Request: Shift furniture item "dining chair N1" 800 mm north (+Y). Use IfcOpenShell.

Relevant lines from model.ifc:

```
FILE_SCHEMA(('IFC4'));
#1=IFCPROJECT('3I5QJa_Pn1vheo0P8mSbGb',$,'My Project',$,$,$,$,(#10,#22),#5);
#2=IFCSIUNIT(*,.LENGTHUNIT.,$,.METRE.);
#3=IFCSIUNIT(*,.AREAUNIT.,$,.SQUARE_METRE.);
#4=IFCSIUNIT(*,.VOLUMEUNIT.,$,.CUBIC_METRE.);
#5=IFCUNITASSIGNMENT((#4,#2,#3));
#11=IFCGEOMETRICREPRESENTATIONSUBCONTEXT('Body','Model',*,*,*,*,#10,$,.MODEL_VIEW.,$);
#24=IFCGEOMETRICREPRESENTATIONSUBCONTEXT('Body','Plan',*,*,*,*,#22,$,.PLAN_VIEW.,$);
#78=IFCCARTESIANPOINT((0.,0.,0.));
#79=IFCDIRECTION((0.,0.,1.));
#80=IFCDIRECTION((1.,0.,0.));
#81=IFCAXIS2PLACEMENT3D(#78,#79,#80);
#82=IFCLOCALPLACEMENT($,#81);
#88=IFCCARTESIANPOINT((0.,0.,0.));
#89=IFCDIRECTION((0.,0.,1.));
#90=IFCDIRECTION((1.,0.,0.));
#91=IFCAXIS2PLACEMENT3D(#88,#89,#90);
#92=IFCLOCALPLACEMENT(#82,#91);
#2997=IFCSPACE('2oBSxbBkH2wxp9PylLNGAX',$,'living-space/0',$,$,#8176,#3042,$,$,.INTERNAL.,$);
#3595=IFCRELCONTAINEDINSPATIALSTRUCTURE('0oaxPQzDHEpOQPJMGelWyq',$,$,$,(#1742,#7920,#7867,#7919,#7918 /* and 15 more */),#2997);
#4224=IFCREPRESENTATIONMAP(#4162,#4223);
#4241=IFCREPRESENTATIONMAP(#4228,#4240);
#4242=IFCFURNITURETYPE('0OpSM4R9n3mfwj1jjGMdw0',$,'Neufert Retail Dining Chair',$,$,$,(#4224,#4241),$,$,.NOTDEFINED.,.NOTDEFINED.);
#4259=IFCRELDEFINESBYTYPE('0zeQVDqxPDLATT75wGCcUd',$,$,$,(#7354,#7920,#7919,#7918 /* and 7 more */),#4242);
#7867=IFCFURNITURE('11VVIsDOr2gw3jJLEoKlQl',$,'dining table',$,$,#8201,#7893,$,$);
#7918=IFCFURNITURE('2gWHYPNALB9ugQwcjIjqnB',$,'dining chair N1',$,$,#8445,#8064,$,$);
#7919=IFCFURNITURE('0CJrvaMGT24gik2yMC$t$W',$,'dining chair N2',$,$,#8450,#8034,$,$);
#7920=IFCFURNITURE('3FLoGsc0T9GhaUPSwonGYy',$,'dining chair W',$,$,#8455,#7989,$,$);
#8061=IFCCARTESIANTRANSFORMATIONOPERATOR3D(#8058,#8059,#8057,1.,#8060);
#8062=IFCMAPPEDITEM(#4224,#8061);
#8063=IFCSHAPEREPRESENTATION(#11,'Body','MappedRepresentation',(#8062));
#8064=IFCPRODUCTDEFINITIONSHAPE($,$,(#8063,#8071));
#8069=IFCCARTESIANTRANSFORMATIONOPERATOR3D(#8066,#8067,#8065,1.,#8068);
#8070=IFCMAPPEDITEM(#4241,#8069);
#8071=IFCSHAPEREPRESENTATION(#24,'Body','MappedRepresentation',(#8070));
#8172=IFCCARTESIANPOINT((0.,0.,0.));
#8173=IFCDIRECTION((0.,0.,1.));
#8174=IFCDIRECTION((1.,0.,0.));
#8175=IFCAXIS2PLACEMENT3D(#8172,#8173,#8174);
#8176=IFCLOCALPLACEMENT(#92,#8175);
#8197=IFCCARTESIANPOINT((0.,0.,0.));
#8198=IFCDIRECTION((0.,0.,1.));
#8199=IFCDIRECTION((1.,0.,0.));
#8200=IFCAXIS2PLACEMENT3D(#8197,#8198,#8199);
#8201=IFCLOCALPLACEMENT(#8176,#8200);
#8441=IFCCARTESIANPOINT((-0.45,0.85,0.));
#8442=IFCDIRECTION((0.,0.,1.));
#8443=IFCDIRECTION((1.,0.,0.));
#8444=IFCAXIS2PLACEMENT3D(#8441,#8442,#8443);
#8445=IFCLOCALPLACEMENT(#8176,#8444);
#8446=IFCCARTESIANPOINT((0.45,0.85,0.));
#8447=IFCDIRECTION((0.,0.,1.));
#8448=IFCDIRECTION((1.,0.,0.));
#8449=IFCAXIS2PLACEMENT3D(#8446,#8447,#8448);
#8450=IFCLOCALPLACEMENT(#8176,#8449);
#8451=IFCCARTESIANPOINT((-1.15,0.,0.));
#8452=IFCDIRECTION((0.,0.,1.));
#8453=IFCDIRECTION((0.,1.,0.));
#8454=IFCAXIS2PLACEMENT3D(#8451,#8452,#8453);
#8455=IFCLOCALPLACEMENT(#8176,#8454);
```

```python
import ifcopenshell
import ifcopenshell.api.geometry
import ifcopenshell.util.placement
import ifcopenshell.util.unit

model = ifcopenshell.open("model.ifc")
unit_scale = ifcopenshell.util.unit.calculate_unit_scale(model)

item = model.by_id(7918)
matrix = ifcopenshell.util.placement.get_local_placement(item.ObjectPlacement)
matrix[1, 3] += 0.8 / unit_scale
ifcopenshell.api.geometry.edit_object_placement(model, product=item, matrix=matrix, is_si=False)

print(ifcopenshell.util.placement.get_local_placement(item.ObjectPlacement).round(3) + 0.0)

model.write("model_edited.ifc")
```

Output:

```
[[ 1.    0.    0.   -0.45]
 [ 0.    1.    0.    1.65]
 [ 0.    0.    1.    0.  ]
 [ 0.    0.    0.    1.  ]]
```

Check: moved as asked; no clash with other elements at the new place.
